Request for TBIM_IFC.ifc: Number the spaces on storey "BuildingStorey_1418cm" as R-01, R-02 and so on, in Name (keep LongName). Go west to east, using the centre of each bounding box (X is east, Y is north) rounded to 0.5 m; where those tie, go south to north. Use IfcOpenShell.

First a look at what the model holds.

```python
import ifcopenshell
import ifcopenshell.util.element
import ifcopenshell.util.placement

model = ifcopenshell.open("TBIM_IFC.ifc")
print(model.schema)
storey = next(s for s in model.by_type("IfcBuildingStorey") if s.Name == "BuildingStorey_1418cm")
spaces = [e for e in ifcopenshell.util.element.get_decomposition(storey) if e.is_a("IfcSpace")]
for e in sorted(spaces, key=lambda e: e.id()):
    origin = ifcopenshell.util.placement.get_local_placement(e.ObjectPlacement)[:3, 3]
    print(e.id(), e.Name, e.LongName, origin.round(2) + 0.0, sep=" | ")
```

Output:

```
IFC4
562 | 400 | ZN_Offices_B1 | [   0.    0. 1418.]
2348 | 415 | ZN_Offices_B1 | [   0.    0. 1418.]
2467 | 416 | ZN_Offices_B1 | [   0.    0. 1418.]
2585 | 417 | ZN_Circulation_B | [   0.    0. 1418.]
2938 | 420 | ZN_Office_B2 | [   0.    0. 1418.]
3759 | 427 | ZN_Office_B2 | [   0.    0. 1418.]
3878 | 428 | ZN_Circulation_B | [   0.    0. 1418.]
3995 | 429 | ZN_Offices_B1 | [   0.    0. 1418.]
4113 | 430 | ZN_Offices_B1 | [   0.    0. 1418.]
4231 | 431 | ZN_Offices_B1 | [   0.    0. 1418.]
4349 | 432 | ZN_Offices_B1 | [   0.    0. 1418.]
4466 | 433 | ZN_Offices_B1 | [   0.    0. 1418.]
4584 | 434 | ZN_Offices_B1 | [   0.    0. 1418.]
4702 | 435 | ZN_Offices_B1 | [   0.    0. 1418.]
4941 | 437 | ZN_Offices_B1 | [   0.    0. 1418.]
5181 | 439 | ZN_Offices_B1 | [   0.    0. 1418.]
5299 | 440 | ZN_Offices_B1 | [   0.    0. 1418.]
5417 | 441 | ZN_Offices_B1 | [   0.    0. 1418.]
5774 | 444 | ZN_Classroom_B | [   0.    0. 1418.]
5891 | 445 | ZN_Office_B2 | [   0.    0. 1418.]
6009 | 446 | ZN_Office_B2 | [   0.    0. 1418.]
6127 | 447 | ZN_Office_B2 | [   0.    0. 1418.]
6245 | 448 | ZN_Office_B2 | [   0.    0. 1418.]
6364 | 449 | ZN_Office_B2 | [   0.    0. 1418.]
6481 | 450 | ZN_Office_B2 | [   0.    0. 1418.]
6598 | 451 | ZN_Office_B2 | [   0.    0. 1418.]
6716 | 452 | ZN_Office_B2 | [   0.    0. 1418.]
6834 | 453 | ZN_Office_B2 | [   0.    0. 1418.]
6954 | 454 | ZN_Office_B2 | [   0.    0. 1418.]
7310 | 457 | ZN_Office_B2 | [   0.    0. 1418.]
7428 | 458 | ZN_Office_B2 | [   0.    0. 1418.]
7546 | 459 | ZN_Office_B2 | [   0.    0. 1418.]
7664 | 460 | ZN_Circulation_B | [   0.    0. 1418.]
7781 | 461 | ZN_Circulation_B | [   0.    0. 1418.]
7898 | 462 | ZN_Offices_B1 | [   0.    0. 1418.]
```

```python
import ifcopenshell
import ifcopenshell.geom
import ifcopenshell.util.element
import ifcopenshell.util.shape

model = ifcopenshell.open("TBIM_IFC.ifc")
settings = ifcopenshell.geom.settings()
settings.set("use-world-coords", True)


def centre(element):
    shape = ifcopenshell.geom.create_shape(settings, element)
    return ifcopenshell.util.shape.get_bbox_centroid(shape.geometry)


storey = next(s for s in model.by_type("IfcBuildingStorey") if s.Name == "BuildingStorey_1418cm")
spaces = [e for e in ifcopenshell.util.element.get_decomposition(storey) if e.is_a("IfcSpace")]

# Insertion points can sit at a corner or the storey origin, so sort by the geometry (in metres).
centres = {e: centre(e) for e in spaces}
spaces.sort(key=lambda e: (round(centres[e][0] / 0.5), centres[e][1]))

for i, e in enumerate(spaces, start=1):
    number = f"R-{i:02d}"
    e.Name = number
    print(e.id(), number)

model.write("TBIM_IFC_rev.ifc")
```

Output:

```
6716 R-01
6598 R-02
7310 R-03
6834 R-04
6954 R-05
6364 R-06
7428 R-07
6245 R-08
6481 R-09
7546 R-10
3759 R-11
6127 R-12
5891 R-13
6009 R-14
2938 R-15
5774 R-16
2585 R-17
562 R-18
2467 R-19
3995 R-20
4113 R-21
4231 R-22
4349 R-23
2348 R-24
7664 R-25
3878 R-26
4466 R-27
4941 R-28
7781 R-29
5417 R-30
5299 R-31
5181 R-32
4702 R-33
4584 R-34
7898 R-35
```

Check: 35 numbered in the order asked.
